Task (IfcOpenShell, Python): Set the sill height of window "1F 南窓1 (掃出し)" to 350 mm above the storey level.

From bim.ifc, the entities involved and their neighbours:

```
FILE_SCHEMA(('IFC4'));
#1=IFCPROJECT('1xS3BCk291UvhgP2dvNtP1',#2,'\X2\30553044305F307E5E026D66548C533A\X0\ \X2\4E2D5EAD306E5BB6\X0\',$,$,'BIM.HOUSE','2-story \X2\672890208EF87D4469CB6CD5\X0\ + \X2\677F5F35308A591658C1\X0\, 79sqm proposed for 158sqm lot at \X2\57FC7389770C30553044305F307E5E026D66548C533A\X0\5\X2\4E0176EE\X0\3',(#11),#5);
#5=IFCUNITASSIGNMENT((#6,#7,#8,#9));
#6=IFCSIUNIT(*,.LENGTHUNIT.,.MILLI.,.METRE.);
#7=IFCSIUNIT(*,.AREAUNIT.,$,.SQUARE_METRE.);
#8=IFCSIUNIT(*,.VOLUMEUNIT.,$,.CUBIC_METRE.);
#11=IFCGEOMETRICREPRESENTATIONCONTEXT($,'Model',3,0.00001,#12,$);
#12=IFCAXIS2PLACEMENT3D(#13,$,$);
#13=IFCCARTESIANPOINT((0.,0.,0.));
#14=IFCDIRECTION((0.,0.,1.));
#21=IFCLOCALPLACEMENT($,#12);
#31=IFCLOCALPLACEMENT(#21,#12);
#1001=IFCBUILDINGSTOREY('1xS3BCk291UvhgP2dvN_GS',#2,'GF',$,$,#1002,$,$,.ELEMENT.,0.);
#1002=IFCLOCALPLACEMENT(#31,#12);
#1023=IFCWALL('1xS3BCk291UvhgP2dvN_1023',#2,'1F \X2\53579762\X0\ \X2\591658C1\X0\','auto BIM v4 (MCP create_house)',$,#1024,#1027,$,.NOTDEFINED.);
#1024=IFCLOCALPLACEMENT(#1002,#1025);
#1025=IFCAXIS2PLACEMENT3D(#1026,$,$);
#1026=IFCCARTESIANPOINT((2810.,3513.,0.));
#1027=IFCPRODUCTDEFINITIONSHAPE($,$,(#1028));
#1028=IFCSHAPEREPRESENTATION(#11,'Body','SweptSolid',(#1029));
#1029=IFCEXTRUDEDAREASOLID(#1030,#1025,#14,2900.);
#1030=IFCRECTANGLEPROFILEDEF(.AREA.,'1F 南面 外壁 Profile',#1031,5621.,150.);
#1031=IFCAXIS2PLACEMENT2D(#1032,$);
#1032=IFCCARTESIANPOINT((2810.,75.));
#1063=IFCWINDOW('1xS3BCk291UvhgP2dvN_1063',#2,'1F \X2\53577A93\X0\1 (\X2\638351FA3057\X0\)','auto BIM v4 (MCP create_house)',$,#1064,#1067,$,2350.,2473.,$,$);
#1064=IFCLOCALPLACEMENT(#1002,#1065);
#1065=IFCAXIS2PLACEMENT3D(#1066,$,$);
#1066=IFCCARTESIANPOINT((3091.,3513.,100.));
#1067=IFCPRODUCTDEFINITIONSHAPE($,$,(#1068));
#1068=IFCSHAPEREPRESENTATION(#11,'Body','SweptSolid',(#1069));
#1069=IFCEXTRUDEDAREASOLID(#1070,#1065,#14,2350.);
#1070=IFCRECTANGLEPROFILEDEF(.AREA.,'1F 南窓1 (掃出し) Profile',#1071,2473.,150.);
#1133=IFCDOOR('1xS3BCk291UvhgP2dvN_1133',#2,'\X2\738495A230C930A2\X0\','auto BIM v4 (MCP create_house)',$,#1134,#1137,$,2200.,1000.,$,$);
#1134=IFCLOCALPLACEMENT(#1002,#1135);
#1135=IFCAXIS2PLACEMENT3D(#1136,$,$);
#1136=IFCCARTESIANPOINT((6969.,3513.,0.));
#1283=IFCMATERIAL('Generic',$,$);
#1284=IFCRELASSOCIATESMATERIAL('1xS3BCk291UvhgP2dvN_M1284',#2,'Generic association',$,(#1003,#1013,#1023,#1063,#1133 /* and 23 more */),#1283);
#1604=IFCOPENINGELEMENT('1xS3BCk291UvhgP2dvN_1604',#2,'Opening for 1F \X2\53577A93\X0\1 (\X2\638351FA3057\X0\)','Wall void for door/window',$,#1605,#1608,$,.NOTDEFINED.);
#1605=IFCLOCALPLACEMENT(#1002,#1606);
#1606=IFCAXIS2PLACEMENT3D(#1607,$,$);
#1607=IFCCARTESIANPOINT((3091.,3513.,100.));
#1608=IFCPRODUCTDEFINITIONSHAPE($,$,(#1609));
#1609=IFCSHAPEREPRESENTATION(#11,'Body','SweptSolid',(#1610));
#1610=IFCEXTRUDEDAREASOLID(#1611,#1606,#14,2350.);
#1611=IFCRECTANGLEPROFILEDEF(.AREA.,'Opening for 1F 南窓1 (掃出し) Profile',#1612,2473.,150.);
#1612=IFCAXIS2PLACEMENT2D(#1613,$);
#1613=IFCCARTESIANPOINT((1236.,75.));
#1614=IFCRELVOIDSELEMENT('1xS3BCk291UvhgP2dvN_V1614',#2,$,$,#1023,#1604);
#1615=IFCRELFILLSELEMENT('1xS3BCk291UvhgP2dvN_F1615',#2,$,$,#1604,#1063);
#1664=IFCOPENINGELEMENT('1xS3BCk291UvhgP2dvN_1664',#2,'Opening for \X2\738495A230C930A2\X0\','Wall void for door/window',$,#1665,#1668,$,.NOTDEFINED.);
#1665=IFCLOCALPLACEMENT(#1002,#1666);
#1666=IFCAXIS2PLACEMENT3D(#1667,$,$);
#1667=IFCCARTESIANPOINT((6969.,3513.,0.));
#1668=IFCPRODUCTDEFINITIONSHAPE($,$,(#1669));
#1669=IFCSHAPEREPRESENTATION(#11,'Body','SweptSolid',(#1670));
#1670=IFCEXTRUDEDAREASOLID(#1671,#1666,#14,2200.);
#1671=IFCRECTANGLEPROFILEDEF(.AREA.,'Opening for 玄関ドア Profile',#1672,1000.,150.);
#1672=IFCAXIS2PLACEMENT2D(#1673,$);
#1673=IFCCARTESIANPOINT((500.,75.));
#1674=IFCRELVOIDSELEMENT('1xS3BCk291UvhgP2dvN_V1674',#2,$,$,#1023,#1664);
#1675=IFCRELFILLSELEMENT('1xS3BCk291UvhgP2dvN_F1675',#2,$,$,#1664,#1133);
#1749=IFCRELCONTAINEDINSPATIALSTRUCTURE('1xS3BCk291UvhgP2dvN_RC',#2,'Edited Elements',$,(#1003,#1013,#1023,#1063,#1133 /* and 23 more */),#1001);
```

```python
import numpy as np
import ifcopenshell
import ifcopenshell.api.geometry
import ifcopenshell.geom
import ifcopenshell.util.element
import ifcopenshell.util.placement
import ifcopenshell.util.shape
import ifcopenshell.util.unit

model = ifcopenshell.open("bim.ifc")
unit_scale = ifcopenshell.util.unit.calculate_unit_scale(model)

window = model.by_guid("1xS3BCk291UvhgP2dvN_1063")
opening = window.FillsVoids[0].RelatingOpeningElement
storey = ifcopenshell.util.element.get_container(window, ifc_class="IfcBuildingStorey")
level = ifcopenshell.util.placement.get_local_placement(storey.ObjectPlacement)[2, 3]

# The opening's origin need not be at the sill, so measure its lowest point.
shape = ifcopenshell.geom.create_shape(ifcopenshell.geom.settings(), opening)
bottom = ifcopenshell.util.shape.get_shape_bottom_elevation(shape, shape.geometry) / unit_scale
dz = level + 0.35 / unit_scale - bottom

shift = np.array([0.0, 0.0, dz])
# The window is not placed relative to its opening, so move both.
for product in (opening, window):
    matrix = ifcopenshell.util.placement.get_local_placement(product.ObjectPlacement)
    matrix[:3, 3] += shift
    ifcopenshell.api.geometry.edit_object_placement(model, product=product, matrix=matrix, is_si=False)

print(f"moved by {dz * unit_scale:+.3f} m")

model.write("bim_v2.ifc")
```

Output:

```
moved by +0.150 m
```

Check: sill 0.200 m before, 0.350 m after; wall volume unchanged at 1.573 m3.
